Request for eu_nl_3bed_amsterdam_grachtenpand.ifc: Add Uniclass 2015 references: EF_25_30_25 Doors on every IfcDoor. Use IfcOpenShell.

First a look at what the model holds.

```python
import ifcopenshell

model = ifcopenshell.open("eu_nl_3bed_amsterdam_grachtenpand.ifc")
print(model.schema)
print("classifications:", [c.Name for c in model.by_type("IfcClassification")])
for ifc_class in ("IfcDoor", "IfcRoof", "IfcStair", "IfcWall", "IfcWindow"):
    print(ifc_class, len(model.by_type(ifc_class)))
```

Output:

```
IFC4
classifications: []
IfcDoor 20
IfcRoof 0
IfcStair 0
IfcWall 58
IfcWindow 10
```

```python
import ifcopenshell
import ifcopenshell.api.classification

model = ifcopenshell.open("eu_nl_3bed_amsterdam_grachtenpand.ifc")

system = ifcopenshell.api.classification.add_classification(model, classification="Uniclass 2015")

codes = {
    "IfcDoor": ("EF_25_30_25", "Doors"),
}
for ifc_class, (code, name) in codes.items():
    products = model.by_type(ifc_class)
    ifcopenshell.api.classification.add_reference(
        model, products=products, classification=system, identification=code, name=name
    )
    print(code, len(products))

model.write("eu_nl_3bed_amsterdam_grachtenpand_rev.ifc")
```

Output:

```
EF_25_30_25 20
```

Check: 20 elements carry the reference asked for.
